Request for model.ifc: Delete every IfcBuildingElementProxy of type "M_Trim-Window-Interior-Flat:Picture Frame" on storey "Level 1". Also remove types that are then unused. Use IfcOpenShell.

First a look at what the model holds.

```python
import ifcopenshell
import ifcopenshell.util.element

model = ifcopenshell.open("model.ifc")
print(model.schema)
storey = next(s for s in model.by_type("IfcBuildingStorey") if s.Name == "Level 1")
proxies = [e for e in ifcopenshell.util.element.get_decomposition(storey) if e.is_a("IfcBuildingElementProxy")]
seen = {}
for e in proxies:
    element_type = ifcopenshell.util.element.get_type(e)
    name = element_type.Name if element_type not in (None, e) else None
    seen[name] = seen.get(name, 0) + 1
for name, count in sorted(seen.items(), key=str):
    print(count, "x", name)
```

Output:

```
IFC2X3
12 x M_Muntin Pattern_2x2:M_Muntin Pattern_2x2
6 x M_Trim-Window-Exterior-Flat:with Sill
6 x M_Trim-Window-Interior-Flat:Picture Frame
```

```python
import ifcopenshell
import ifcopenshell.api.root
import ifcopenshell.util.element

model = ifcopenshell.open("model.ifc")

storey = next(s for s in model.by_type("IfcBuildingStorey") if s.Name == "Level 1")
proxies = [e for e in ifcopenshell.util.element.get_decomposition(storey) if e.is_a("IfcBuildingElementProxy")]
targets = [e for e in proxies if (t := ifcopenshell.util.element.get_type(e)) not in (None, e) and t.Name == "M_Trim-Window-Interior-Flat:Picture Frame"]
types = {ifcopenshell.util.element.get_type(e) for e in targets} - {None, *targets}

for e in targets:
    ifcopenshell.api.root.remove_product(model, product=e)
print(len(targets), "removed")

unused = [t for t in types if not ifcopenshell.util.element.get_types(t)]
for t in unused:
    ifcopenshell.api.root.remove_product(model, product=t)
print(len(unused), "unused types removed")

model.write("model-out.ifc")
```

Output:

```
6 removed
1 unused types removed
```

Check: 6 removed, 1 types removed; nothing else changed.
